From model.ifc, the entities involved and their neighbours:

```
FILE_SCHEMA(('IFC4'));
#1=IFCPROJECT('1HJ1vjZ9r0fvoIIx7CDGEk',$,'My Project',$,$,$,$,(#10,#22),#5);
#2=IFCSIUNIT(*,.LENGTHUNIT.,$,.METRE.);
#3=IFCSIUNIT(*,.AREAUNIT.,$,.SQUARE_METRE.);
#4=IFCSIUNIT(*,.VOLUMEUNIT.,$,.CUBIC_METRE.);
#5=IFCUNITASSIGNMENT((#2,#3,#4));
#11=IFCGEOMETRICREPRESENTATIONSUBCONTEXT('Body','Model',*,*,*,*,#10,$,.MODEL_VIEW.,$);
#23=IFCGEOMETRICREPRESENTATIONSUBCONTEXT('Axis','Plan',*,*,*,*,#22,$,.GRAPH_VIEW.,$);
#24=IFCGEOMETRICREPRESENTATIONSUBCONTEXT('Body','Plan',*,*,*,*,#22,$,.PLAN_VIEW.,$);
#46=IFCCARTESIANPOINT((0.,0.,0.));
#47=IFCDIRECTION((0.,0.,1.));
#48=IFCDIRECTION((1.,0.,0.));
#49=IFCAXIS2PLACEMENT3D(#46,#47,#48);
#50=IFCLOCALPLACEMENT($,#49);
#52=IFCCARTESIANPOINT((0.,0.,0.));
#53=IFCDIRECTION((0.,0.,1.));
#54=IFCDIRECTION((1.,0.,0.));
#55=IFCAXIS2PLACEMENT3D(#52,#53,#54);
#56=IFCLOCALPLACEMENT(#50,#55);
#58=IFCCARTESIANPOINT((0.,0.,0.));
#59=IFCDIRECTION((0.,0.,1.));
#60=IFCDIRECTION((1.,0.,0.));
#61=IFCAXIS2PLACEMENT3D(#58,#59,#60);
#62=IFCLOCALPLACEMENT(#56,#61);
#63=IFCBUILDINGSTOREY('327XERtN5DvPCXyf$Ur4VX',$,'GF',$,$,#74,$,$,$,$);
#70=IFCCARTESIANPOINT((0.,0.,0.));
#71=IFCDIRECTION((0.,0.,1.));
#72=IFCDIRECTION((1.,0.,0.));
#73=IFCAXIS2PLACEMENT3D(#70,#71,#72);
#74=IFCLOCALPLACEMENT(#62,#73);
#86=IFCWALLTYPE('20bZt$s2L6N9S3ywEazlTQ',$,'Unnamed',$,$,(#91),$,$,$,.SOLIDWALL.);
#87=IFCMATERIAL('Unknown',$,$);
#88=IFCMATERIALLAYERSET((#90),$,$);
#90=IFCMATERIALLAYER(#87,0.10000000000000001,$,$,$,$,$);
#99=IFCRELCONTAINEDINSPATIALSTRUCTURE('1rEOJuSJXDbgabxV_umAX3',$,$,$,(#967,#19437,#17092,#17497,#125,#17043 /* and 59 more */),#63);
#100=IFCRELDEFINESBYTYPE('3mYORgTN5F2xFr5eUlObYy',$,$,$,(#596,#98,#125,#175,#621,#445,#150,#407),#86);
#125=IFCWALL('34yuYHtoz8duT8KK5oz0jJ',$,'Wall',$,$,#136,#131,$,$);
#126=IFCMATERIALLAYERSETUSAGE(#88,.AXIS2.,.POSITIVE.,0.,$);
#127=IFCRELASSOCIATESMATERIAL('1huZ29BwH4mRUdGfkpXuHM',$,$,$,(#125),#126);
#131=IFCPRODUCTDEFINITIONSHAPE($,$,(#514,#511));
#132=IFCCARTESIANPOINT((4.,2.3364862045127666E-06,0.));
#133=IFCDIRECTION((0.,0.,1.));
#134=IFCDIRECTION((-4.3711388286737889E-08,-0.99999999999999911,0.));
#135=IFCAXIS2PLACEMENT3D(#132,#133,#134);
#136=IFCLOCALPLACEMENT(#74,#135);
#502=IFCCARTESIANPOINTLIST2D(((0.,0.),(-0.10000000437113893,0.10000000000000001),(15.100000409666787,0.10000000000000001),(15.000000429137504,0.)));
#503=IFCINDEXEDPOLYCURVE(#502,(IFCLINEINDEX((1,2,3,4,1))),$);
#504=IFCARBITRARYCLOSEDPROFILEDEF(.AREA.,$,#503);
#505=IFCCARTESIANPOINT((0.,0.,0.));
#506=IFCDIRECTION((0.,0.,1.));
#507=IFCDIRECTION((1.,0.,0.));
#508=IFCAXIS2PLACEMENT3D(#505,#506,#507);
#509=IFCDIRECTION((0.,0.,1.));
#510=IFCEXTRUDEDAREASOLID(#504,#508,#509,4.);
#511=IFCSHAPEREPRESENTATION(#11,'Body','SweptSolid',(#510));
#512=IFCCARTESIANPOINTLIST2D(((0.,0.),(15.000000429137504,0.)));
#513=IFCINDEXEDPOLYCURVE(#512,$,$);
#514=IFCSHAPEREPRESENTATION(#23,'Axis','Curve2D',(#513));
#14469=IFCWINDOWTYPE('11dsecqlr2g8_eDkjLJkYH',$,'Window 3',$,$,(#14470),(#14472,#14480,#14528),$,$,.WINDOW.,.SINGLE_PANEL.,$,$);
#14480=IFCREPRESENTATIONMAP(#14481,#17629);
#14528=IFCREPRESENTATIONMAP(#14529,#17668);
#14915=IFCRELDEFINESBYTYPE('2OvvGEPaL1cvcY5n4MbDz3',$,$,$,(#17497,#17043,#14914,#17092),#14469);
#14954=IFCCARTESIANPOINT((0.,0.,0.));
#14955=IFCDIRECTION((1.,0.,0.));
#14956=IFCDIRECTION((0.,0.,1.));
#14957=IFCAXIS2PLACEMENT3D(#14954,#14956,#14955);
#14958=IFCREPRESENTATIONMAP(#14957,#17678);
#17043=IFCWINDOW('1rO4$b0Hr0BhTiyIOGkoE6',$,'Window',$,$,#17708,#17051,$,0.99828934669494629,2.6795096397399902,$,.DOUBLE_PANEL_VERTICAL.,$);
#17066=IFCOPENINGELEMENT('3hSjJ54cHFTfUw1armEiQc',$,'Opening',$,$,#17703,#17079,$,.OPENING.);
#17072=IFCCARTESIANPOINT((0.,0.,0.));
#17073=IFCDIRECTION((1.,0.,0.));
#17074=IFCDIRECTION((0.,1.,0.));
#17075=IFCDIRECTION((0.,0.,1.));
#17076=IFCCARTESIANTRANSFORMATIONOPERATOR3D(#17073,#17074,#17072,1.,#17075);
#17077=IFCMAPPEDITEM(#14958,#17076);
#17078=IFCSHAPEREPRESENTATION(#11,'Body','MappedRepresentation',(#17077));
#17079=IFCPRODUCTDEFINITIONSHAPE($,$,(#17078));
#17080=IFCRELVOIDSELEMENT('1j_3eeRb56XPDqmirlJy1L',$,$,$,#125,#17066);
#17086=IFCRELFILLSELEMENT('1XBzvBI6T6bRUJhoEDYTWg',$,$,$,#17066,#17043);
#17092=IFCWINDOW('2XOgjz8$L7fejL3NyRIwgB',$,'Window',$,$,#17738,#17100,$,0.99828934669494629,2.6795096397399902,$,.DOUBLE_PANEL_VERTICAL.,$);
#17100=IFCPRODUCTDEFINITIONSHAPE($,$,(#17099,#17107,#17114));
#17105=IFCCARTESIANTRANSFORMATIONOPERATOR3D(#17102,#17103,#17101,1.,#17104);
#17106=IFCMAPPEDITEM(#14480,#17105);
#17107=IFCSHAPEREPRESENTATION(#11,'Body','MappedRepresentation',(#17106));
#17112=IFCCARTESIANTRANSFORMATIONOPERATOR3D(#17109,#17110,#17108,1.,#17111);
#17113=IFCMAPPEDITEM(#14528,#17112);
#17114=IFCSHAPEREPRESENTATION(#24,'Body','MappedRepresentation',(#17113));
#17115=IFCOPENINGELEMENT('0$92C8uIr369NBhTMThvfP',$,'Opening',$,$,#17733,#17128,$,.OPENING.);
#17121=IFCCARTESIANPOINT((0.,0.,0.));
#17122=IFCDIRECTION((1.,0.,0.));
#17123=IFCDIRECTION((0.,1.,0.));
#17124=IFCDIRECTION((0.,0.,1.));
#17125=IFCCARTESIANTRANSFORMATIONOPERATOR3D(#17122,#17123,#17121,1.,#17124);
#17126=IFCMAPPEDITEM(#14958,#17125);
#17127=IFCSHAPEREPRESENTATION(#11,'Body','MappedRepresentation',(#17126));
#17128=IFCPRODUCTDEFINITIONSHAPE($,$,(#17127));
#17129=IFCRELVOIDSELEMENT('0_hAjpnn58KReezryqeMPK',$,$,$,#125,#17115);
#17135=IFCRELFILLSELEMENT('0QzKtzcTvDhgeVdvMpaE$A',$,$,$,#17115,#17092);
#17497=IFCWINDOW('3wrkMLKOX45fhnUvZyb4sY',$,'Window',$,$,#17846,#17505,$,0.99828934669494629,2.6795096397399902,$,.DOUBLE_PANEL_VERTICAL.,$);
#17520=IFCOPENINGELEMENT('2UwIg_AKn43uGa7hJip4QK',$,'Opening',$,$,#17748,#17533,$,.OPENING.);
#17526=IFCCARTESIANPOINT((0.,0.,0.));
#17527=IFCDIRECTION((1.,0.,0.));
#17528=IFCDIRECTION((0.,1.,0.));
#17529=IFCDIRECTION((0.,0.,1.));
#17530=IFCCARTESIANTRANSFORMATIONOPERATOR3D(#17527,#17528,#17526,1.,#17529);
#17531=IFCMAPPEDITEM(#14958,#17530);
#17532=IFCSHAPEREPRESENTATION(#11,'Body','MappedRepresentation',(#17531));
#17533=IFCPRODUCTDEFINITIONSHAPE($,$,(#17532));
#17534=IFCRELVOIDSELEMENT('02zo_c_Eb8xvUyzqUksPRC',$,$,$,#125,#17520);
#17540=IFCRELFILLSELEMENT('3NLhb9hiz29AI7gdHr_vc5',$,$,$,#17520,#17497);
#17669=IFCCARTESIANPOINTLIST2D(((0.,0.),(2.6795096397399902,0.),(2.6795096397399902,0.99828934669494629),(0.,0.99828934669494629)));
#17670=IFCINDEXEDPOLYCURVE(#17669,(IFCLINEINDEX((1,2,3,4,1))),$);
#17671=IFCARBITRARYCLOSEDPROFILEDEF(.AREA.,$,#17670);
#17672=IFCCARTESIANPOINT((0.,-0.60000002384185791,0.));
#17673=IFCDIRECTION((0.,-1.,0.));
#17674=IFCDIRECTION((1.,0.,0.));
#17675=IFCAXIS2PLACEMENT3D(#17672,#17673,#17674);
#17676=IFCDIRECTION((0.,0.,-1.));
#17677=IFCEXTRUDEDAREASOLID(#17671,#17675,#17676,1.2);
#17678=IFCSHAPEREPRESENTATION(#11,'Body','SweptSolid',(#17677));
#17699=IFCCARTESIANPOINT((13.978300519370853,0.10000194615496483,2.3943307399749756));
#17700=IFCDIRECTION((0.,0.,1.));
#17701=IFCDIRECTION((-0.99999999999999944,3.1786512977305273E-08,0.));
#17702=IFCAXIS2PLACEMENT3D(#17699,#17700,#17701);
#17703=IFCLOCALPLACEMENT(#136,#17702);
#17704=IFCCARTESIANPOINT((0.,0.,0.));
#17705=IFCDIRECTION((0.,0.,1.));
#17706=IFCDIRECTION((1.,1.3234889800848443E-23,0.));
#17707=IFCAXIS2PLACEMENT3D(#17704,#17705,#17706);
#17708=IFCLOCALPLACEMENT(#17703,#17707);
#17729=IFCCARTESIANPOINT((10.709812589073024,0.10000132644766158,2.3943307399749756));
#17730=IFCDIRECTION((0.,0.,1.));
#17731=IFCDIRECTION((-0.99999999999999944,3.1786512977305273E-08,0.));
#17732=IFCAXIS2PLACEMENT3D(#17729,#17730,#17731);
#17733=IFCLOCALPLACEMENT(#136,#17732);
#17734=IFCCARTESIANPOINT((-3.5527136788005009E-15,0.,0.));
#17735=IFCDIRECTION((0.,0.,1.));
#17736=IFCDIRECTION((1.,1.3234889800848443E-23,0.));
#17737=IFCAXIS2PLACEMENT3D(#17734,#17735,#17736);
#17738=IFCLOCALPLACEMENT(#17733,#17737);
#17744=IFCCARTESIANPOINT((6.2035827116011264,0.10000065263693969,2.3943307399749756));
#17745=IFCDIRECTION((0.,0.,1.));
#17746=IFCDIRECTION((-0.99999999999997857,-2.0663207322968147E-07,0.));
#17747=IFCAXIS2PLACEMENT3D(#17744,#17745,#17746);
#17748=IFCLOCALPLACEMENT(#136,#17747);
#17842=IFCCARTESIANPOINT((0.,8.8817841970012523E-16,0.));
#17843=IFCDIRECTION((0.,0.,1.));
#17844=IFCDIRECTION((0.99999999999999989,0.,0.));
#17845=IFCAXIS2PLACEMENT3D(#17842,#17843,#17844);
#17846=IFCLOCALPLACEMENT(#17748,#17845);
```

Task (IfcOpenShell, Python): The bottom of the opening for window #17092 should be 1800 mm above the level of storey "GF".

```python
import numpy as np
import ifcopenshell
import ifcopenshell.api.geometry
import ifcopenshell.geom
import ifcopenshell.util.element
import ifcopenshell.util.placement
import ifcopenshell.util.shape
import ifcopenshell.util.unit

model = ifcopenshell.open("model.ifc")
unit_scale = ifcopenshell.util.unit.calculate_unit_scale(model)

window = model.by_guid("2XOgjz8$L7fejL3NyRIwgB")
opening = window.FillsVoids[0].RelatingOpeningElement
storey = ifcopenshell.util.element.get_container(window, ifc_class="IfcBuildingStorey")
level = ifcopenshell.util.placement.get_local_placement(storey.ObjectPlacement)[2, 3]

# The opening's origin need not be at the sill, so measure its lowest point.
shape = ifcopenshell.geom.create_shape(ifcopenshell.geom.settings(), opening)
bottom = ifcopenshell.util.shape.get_shape_bottom_elevation(shape, shape.geometry) / unit_scale
dz = level + 1.8 / unit_scale - bottom

shift = np.array([0.0, 0.0, dz])
# The window is placed relative to its opening, so it follows when the opening moves.
matrix = ifcopenshell.util.placement.get_local_placement(opening.ObjectPlacement)
matrix[:3, 3] += shift
ifcopenshell.api.geometry.edit_object_placement(
    model, product=opening, matrix=matrix, is_si=False, should_transform_children=True
)

print(f"moved by {dz * unit_scale:+.3f} m")

model.write("model_rev.ifc")
```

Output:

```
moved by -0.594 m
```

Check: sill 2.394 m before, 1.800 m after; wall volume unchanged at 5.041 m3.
